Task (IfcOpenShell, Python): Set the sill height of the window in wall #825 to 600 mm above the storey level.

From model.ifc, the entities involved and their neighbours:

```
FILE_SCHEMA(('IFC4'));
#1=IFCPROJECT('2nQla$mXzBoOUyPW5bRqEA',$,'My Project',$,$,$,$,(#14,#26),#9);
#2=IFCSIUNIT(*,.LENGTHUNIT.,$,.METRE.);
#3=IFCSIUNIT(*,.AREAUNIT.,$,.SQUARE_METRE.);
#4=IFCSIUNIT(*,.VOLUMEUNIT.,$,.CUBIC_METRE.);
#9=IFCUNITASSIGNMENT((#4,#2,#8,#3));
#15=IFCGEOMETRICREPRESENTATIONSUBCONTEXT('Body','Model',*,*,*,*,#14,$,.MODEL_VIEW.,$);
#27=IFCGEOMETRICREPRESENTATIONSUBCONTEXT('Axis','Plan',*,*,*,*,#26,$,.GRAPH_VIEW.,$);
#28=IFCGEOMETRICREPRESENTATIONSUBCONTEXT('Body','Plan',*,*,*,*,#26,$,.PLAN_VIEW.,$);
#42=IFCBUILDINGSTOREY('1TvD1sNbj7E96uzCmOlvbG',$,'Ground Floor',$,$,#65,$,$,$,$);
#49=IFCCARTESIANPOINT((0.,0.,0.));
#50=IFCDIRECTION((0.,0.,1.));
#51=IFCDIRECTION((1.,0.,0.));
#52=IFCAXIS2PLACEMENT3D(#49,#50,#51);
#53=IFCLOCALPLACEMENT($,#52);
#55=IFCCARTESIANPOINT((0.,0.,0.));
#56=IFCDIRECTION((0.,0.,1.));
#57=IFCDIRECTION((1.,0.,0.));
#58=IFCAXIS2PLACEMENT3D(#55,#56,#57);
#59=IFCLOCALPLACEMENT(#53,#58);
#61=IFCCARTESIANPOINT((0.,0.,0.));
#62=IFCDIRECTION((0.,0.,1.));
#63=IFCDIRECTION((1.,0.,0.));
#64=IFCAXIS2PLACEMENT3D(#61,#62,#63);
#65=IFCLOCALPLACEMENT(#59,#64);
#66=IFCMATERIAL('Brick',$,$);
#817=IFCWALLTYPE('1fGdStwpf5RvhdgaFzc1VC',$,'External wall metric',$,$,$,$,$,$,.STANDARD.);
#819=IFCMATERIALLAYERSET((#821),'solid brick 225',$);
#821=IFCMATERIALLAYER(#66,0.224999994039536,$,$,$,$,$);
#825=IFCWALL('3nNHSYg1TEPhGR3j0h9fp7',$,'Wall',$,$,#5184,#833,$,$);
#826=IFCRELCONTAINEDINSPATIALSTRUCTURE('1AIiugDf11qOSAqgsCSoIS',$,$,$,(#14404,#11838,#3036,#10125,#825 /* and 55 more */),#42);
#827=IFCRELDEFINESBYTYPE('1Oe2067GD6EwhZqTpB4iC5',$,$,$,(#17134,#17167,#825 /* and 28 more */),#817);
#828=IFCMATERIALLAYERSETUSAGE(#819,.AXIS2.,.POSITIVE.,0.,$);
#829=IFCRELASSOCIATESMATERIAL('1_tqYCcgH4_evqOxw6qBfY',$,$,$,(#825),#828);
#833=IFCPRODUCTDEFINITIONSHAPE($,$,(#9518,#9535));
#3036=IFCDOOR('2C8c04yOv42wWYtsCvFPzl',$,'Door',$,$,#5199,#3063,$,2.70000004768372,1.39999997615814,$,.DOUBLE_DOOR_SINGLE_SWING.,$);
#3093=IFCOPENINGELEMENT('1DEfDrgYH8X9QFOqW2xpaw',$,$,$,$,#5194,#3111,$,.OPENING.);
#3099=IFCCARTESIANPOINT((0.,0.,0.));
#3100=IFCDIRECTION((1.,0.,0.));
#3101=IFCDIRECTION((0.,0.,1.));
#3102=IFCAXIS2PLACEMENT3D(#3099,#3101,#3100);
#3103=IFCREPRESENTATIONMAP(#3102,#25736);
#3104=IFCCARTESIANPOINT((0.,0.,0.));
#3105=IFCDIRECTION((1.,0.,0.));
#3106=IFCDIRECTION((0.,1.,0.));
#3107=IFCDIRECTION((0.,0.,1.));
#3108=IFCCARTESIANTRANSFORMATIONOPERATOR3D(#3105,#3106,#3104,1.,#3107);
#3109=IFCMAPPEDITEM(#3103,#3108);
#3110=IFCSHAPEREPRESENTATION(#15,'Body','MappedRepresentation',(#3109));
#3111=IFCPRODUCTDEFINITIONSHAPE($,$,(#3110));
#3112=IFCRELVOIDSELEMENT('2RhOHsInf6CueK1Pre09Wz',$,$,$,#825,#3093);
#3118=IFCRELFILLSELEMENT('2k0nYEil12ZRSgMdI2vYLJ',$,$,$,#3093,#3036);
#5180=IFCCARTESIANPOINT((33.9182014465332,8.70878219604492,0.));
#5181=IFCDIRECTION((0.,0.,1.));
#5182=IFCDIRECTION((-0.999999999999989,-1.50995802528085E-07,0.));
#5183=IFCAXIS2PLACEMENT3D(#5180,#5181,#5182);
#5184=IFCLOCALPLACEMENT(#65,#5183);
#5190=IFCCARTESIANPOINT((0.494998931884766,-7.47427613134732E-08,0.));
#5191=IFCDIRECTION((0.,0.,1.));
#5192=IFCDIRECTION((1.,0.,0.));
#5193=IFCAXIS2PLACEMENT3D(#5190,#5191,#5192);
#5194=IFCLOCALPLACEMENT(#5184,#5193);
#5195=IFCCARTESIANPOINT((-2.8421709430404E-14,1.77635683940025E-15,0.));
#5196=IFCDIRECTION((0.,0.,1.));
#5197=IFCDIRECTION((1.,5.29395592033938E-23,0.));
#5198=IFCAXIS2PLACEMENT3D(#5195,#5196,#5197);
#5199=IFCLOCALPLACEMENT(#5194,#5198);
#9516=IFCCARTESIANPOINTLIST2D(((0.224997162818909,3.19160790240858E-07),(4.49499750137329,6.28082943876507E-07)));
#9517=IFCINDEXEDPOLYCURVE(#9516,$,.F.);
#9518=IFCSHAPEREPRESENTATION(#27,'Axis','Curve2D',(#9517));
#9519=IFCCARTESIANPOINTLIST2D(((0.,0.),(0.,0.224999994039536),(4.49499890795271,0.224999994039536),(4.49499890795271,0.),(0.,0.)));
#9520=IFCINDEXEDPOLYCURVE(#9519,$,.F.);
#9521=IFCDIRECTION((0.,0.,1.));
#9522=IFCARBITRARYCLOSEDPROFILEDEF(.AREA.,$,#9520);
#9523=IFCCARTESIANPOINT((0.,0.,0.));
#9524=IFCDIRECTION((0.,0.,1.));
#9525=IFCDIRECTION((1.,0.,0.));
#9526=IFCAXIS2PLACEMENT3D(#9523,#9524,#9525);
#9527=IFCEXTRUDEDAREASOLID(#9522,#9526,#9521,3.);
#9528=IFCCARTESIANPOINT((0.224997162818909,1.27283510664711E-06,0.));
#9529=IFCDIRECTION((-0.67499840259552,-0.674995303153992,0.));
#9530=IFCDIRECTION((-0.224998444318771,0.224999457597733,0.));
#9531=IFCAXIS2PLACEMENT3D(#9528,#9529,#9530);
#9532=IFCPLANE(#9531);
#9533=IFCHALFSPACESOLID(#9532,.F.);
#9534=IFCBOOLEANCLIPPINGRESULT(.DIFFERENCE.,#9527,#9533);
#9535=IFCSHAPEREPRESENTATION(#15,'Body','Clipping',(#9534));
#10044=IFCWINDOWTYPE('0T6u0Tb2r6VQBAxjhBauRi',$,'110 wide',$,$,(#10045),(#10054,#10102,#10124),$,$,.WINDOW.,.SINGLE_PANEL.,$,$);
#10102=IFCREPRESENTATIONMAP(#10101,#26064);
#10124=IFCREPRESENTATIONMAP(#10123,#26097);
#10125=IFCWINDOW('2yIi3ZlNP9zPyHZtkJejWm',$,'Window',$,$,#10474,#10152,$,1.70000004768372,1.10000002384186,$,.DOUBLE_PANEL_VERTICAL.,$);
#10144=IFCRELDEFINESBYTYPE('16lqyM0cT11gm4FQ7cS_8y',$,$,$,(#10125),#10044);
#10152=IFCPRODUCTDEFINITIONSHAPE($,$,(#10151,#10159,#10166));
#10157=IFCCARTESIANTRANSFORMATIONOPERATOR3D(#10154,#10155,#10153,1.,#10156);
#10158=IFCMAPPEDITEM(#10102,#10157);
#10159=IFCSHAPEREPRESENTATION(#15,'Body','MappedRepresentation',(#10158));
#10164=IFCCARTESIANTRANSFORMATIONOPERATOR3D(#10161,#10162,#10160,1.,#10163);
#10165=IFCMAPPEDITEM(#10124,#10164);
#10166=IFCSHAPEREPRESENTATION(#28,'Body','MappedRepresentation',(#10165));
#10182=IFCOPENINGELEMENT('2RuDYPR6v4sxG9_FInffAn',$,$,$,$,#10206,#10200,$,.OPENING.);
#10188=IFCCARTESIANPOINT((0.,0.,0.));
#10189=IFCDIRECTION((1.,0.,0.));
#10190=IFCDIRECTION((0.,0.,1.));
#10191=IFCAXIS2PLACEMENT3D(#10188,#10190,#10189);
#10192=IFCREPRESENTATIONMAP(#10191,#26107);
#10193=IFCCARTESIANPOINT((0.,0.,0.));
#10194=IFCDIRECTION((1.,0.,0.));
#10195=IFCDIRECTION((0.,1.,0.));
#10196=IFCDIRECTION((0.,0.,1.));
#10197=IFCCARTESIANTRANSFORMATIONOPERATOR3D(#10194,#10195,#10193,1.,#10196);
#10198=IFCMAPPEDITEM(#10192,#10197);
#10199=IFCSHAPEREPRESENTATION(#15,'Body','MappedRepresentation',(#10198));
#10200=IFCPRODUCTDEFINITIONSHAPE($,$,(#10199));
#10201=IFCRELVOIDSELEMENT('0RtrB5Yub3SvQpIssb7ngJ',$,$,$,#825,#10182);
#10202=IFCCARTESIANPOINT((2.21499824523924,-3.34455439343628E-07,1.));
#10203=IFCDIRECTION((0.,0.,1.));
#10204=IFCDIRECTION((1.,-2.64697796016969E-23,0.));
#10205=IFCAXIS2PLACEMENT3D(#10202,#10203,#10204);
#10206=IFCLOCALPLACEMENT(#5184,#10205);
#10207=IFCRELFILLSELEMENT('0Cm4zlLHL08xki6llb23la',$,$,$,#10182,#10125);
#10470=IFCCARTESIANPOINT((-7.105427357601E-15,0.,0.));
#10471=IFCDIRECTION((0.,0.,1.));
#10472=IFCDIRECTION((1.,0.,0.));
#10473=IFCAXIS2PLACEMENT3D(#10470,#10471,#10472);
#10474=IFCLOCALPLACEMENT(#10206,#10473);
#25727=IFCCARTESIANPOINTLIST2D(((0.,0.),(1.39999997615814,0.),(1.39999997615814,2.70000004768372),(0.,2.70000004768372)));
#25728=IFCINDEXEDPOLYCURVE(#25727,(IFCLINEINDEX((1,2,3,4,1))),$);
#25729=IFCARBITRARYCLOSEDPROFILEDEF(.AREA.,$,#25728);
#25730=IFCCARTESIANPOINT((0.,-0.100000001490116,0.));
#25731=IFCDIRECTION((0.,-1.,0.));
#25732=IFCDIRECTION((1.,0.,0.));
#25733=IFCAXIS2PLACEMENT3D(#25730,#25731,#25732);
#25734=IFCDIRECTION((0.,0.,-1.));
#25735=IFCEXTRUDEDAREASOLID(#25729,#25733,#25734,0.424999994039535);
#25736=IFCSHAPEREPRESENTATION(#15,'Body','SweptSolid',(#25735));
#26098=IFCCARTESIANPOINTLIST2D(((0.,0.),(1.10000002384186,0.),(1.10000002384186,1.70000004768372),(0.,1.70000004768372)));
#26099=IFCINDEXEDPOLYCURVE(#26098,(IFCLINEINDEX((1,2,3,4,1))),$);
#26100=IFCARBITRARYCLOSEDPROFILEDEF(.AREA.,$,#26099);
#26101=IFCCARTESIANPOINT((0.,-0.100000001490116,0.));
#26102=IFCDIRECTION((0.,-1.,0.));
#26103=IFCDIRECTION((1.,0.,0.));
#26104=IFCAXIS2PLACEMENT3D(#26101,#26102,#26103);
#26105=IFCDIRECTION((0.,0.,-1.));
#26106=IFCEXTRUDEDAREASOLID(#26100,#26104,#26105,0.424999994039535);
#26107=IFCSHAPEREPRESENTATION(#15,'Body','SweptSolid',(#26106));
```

```python
import numpy as np
import ifcopenshell
import ifcopenshell.api.geometry
import ifcopenshell.geom
import ifcopenshell.util.element
import ifcopenshell.util.placement
import ifcopenshell.util.shape
import ifcopenshell.util.unit

model = ifcopenshell.open("model.ifc")
unit_scale = ifcopenshell.util.unit.calculate_unit_scale(model)

window = model.by_guid("2yIi3ZlNP9zPyHZtkJejWm")
opening = window.FillsVoids[0].RelatingOpeningElement
storey = ifcopenshell.util.element.get_container(window, ifc_class="IfcBuildingStorey")
level = ifcopenshell.util.placement.get_local_placement(storey.ObjectPlacement)[2, 3]

# The opening's origin need not be at the sill, so measure its lowest point.
shape = ifcopenshell.geom.create_shape(ifcopenshell.geom.settings(), opening)
bottom = ifcopenshell.util.shape.get_shape_bottom_elevation(shape, shape.geometry) / unit_scale
dz = level + 0.6 - bottom

shift = np.array([0.0, 0.0, dz])
# The window is placed relative to its opening, so it follows when the opening moves.
matrix = ifcopenshell.util.placement.get_local_placement(opening.ObjectPlacement)
matrix[:3, 3] += shift
ifcopenshell.api.geometry.edit_object_placement(
    model, product=opening, matrix=matrix, is_si=False, should_transform_children=True
)

print(f"moved by {dz * unit_scale:+.3f} m")

model.write("model_rev.ifc")
```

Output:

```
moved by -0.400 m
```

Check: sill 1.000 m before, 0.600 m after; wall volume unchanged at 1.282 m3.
